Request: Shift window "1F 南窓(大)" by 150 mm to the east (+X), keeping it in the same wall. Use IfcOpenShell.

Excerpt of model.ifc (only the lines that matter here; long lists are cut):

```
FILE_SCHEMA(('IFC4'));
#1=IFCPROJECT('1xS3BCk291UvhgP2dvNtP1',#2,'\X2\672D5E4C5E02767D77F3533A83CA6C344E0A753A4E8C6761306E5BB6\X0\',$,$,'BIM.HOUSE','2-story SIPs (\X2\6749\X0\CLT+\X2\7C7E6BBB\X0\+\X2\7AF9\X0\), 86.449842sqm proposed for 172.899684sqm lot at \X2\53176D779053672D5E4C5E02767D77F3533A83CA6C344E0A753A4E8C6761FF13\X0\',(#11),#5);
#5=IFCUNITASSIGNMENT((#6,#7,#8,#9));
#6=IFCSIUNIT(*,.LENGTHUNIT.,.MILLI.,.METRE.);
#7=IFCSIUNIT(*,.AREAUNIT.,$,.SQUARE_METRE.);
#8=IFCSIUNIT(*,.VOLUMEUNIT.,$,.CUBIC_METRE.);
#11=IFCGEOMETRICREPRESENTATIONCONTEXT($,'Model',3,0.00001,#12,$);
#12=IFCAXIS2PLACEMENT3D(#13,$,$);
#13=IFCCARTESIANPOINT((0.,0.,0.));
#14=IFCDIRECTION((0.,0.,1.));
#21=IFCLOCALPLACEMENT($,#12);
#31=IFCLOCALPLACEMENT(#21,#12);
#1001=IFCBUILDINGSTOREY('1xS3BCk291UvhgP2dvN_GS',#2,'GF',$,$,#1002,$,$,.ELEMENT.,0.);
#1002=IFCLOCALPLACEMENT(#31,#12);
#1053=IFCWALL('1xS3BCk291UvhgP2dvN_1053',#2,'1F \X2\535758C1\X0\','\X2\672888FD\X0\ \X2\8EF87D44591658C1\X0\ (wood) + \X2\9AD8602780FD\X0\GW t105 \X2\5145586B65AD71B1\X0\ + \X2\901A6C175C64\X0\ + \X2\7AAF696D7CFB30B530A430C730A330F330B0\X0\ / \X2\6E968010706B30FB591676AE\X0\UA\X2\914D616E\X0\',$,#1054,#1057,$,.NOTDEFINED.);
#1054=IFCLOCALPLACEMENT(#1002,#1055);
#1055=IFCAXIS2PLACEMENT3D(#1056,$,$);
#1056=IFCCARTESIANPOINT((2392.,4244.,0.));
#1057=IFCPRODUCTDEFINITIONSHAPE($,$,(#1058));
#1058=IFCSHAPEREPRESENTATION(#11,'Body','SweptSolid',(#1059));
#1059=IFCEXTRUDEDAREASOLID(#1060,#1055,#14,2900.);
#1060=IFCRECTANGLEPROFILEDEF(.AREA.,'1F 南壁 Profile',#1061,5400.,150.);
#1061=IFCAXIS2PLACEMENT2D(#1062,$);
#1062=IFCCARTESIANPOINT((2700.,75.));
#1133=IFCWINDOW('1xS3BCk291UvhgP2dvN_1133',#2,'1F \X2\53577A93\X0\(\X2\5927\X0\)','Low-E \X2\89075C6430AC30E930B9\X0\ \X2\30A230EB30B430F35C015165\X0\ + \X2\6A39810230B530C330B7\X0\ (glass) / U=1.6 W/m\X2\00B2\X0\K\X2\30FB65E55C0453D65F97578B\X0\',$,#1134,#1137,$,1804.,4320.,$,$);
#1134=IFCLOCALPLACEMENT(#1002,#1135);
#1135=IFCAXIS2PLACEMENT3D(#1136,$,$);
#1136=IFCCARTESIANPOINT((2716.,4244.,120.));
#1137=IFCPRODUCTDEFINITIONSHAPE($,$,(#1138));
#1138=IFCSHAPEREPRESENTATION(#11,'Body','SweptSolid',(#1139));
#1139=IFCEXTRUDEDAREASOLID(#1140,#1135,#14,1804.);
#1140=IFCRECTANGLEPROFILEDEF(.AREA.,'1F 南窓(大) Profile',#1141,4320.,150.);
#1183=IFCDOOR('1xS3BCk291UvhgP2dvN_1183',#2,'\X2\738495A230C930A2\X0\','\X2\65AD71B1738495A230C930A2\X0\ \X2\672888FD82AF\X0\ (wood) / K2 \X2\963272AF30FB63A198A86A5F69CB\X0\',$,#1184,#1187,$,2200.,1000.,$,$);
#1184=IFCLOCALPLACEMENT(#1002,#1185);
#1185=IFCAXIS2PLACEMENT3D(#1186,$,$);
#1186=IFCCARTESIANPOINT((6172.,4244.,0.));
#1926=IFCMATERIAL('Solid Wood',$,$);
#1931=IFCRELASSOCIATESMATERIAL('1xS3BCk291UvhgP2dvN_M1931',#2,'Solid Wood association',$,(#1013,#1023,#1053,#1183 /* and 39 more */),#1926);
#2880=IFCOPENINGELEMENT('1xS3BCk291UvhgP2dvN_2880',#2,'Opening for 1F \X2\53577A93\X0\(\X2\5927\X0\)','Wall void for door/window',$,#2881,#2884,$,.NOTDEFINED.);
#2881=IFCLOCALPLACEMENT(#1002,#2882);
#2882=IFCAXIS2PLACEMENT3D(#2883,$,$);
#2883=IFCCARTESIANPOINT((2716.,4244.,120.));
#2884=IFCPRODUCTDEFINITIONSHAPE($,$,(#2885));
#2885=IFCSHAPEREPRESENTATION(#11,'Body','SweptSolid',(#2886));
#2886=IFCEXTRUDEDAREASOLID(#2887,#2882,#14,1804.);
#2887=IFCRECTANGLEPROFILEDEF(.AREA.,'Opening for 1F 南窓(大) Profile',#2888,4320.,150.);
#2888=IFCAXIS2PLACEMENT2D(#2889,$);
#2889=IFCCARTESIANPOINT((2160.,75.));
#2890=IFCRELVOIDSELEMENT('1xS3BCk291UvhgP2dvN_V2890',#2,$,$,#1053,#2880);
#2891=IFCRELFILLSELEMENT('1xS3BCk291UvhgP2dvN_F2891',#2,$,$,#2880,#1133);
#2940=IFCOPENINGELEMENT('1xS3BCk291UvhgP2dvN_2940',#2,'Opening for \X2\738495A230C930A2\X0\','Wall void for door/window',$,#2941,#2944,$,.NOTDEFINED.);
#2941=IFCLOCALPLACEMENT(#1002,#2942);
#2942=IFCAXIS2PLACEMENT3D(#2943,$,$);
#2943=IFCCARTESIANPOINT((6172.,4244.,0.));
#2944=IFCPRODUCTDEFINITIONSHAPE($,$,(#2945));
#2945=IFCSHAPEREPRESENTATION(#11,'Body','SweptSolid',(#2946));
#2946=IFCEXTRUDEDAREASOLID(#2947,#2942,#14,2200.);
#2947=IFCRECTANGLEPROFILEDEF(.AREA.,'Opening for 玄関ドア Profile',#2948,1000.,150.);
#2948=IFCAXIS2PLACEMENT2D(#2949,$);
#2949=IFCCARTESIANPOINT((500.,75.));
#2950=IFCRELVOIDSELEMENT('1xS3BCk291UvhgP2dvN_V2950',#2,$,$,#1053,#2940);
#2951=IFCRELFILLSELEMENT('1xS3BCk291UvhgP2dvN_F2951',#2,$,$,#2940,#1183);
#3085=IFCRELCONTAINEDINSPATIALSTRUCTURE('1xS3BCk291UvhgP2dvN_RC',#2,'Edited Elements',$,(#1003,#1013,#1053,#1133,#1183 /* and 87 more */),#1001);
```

```python
import ifcopenshell
import ifcopenshell.api.geometry
import ifcopenshell.util.placement
import ifcopenshell.util.unit

model = ifcopenshell.open("model.ifc")
unit_scale = ifcopenshell.util.unit.calculate_unit_scale(model)

window = model.by_guid("1xS3BCk291UvhgP2dvN_1133")
opening = window.FillsVoids[0].RelatingOpeningElement
wall = opening.VoidsElements[0].RelatingBuildingElement

wall_matrix = ifcopenshell.util.placement.get_local_placement(wall.ObjectPlacement)
shift = wall_matrix[:3, 0] * 0.15 / unit_scale
before = ifcopenshell.util.placement.get_local_placement(window.ObjectPlacement)[:3, 3].copy()

# The window is not placed relative to its opening, so move both.
for product in (opening, window):
    matrix = ifcopenshell.util.placement.get_local_placement(product.ObjectPlacement)
    matrix[:3, 3] += shift
    ifcopenshell.api.geometry.edit_object_placement(model, product=product, matrix=matrix, is_si=False)

after = ifcopenshell.util.placement.get_local_placement(window.ObjectPlacement)[:3, 3]
print("window moved by", (after - before).round(3) + 0.0)

model.write("model_updated.ifc")
```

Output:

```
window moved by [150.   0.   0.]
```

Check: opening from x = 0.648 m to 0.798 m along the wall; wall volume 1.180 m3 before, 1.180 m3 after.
